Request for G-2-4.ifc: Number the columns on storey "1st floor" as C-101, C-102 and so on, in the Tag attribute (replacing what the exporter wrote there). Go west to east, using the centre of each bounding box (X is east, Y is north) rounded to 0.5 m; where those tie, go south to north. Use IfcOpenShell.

First a look at what the model holds.

```python
import ifcopenshell
import ifcopenshell.util.element
import ifcopenshell.util.placement

model = ifcopenshell.open("G-2-4.ifc")
print(model.schema)
storey = next(s for s in model.by_type("IfcBuildingStorey") if s.Name == "1st floor")
columns = [e for e in ifcopenshell.util.element.get_decomposition(storey) if e.is_a("IfcColumn")]
for e in sorted(columns, key=lambda e: e.id()):
    origin = ifcopenshell.util.placement.get_local_placement(e.ObjectPlacement)[:3, 3]
    print(e.id(), e.Tag, e.Name, origin.round(2) + 0.0, sep=" | ")
```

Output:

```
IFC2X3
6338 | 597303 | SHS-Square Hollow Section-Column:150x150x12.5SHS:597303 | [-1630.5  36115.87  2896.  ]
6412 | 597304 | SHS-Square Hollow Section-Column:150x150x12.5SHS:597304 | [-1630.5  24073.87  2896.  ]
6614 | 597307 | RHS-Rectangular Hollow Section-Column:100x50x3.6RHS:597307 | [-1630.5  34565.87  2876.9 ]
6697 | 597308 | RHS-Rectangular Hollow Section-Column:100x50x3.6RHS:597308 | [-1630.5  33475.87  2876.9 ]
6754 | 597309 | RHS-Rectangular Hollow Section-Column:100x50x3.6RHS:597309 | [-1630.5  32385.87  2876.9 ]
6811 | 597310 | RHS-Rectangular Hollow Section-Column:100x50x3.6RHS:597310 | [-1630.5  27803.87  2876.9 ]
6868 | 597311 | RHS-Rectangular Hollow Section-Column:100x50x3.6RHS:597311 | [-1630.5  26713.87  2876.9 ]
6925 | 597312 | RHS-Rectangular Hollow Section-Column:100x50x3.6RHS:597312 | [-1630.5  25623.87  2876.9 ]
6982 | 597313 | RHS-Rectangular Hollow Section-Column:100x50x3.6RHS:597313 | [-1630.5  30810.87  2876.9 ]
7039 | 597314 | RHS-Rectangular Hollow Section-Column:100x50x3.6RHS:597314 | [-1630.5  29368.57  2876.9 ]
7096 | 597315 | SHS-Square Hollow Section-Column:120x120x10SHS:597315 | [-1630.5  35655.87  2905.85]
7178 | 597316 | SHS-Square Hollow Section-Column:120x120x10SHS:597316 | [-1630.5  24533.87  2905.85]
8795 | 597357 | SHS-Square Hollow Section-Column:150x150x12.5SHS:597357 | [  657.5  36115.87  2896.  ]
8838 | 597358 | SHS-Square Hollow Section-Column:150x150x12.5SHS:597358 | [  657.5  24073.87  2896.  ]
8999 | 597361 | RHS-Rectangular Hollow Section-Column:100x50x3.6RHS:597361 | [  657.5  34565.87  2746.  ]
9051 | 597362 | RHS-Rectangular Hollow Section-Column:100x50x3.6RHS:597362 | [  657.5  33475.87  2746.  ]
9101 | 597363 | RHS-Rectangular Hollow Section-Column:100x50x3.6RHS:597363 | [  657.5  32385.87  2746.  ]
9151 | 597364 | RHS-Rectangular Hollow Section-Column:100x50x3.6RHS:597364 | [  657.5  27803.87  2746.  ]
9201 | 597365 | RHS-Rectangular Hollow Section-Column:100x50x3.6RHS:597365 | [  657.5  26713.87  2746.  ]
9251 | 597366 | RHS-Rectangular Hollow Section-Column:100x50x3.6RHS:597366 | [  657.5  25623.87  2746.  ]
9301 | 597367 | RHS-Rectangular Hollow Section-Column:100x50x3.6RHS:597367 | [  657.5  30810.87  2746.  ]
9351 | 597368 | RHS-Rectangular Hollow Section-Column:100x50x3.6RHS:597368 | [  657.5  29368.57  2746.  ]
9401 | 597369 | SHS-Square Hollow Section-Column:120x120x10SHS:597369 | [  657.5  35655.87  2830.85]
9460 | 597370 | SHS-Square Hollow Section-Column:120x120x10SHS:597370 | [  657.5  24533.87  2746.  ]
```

```python
import ifcopenshell
import ifcopenshell.geom
import ifcopenshell.util.element
import ifcopenshell.util.shape

model = ifcopenshell.open("G-2-4.ifc")
settings = ifcopenshell.geom.settings()
settings.set("use-world-coords", True)


def centre(element):
    shape = ifcopenshell.geom.create_shape(settings, element)
    return ifcopenshell.util.shape.get_bbox_centroid(shape.geometry)


storey = next(s for s in model.by_type("IfcBuildingStorey") if s.Name == "1st floor")
columns = [e for e in ifcopenshell.util.element.get_decomposition(storey) if e.is_a("IfcColumn")]

# Insertion points can sit at a corner or the storey origin, so sort by the geometry (in metres).
centres = {e: centre(e) for e in columns}
columns.sort(key=lambda e: (round(centres[e][0] / 0.5), centres[e][1]))

for i, e in enumerate(columns, start=1):
    number = f"C-1{i:02d}"
    e.Tag = number
    print(e.id(), number)

model.write("G-2-4_rev.ifc")
```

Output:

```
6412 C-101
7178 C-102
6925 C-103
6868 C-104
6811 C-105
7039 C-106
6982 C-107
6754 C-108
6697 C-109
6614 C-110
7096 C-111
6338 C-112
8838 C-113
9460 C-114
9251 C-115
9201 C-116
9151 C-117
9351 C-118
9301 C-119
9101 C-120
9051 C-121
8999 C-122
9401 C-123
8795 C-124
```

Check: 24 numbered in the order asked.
